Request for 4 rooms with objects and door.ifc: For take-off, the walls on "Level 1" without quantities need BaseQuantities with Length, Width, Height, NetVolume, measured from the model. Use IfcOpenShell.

First a look at what the model holds.

```python
import ifcopenshell
import ifcopenshell.util.element
import ifcopenshell.util.unit

model = ifcopenshell.open("4 rooms with objects and door.ifc")
print(model.schema)
for unit_type in ("LENGTHUNIT", "AREAUNIT", "VOLUMEUNIT"):
    print(unit_type, ifcopenshell.util.unit.calculate_unit_scale(model, unit_type))
storey = next(s for s in model.by_type("IfcBuildingStorey") if s.Name == "Level 1")
walls = [e for e in ifcopenshell.util.element.get_decomposition(storey) if e.is_a("IfcWall")]
for e in sorted(walls, key=lambda e: e.id()):
    print(e.id(), e.is_a(), e.Name, list(ifcopenshell.util.element.get_psets(e, qtos_only=True)), sep=" | ")
```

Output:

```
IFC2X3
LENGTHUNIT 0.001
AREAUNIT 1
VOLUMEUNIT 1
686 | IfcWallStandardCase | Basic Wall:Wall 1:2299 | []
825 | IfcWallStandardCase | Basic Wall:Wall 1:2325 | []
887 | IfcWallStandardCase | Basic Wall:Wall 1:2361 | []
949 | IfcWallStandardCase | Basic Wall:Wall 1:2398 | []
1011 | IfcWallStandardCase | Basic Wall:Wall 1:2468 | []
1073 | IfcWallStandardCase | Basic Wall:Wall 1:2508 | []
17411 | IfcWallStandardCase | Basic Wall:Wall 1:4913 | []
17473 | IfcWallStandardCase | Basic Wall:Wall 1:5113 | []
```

```python
import ifcopenshell
import ifcopenshell.api.pset
import ifcopenshell.geom
import ifcopenshell.util.element
import ifcopenshell.util.shape
import ifcopenshell.util.unit

model = ifcopenshell.open("4 rooms with objects and door.ifc")
unit_scale = ifcopenshell.util.unit.calculate_unit_scale(model)
volume_scale = ifcopenshell.util.unit.calculate_unit_scale(model, "VOLUMEUNIT")
settings = ifcopenshell.geom.settings()

storey = next(s for s in model.by_type("IfcBuildingStorey") if s.Name == "Level 1")
walls = [e for e in ifcopenshell.util.element.get_decomposition(storey) if e.is_a("IfcWall")]

for e in sorted(walls, key=lambda e: e.id()):
    if ifcopenshell.util.element.get_psets(e, qtos_only=True, should_inherit=False):
        continue
    # Geometry comes back in metres, in the element's own axes.
    shape = ifcopenshell.geom.create_shape(settings, e)
    values = {
        "Length": ifcopenshell.util.shape.get_x(shape.geometry) / unit_scale,
        "Width": ifcopenshell.util.shape.get_y(shape.geometry) / unit_scale,
        "Height": ifcopenshell.util.shape.get_z(shape.geometry) / unit_scale,
        "NetVolume": ifcopenshell.util.shape.get_volume(shape.geometry) / volume_scale,
    }
    qto = ifcopenshell.api.pset.add_qto(model, product=e, name="BaseQuantities")
    ifcopenshell.api.pset.edit_qto(model, qto=qto, properties=values)
    print(e.id(), {k: round(v, 3) for k, v in values.items()})

model.write("4 rooms with objects and door_v2.ifc")
```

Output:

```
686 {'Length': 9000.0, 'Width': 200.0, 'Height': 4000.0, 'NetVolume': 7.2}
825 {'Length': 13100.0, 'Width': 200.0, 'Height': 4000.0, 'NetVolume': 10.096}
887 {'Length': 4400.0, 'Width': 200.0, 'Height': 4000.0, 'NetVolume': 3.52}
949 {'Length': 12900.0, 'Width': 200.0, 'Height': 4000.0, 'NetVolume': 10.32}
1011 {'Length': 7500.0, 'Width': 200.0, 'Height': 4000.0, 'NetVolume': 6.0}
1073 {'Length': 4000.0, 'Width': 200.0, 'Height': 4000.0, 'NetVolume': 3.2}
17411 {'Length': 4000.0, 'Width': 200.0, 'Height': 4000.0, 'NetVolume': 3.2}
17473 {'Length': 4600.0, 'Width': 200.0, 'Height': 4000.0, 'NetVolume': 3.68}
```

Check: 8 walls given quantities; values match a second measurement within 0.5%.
